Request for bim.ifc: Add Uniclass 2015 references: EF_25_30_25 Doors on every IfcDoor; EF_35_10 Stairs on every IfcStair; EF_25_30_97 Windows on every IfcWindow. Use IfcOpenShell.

First a look at what the model holds.

```python
import ifcopenshell

model = ifcopenshell.open("bim.ifc")
print(model.schema)
print("classifications:", [c.Name for c in model.by_type("IfcClassification")])
for ifc_class in ("IfcDoor", "IfcRoof", "IfcStair", "IfcWall", "IfcWindow"):
    print(ifc_class, len(model.by_type(ifc_class)))
```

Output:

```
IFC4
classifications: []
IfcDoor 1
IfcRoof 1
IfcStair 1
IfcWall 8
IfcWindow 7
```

```python
import ifcopenshell
import ifcopenshell.api.classification

model = ifcopenshell.open("bim.ifc")

system = ifcopenshell.api.classification.add_classification(model, classification="Uniclass 2015")

codes = {
    "IfcDoor": ("EF_25_30_25", "Doors"),
    "IfcStair": ("EF_35_10", "Stairs"),
    "IfcWindow": ("EF_25_30_97", "Windows"),
}
for ifc_class, (code, name) in codes.items():
    products = model.by_type(ifc_class)
    ifcopenshell.api.classification.add_reference(
        model, products=products, classification=system, identification=code, name=name
    )
    print(code, len(products))

model.write("bim_updated.ifc")
```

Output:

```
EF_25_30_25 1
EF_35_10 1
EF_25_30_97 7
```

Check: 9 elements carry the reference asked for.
